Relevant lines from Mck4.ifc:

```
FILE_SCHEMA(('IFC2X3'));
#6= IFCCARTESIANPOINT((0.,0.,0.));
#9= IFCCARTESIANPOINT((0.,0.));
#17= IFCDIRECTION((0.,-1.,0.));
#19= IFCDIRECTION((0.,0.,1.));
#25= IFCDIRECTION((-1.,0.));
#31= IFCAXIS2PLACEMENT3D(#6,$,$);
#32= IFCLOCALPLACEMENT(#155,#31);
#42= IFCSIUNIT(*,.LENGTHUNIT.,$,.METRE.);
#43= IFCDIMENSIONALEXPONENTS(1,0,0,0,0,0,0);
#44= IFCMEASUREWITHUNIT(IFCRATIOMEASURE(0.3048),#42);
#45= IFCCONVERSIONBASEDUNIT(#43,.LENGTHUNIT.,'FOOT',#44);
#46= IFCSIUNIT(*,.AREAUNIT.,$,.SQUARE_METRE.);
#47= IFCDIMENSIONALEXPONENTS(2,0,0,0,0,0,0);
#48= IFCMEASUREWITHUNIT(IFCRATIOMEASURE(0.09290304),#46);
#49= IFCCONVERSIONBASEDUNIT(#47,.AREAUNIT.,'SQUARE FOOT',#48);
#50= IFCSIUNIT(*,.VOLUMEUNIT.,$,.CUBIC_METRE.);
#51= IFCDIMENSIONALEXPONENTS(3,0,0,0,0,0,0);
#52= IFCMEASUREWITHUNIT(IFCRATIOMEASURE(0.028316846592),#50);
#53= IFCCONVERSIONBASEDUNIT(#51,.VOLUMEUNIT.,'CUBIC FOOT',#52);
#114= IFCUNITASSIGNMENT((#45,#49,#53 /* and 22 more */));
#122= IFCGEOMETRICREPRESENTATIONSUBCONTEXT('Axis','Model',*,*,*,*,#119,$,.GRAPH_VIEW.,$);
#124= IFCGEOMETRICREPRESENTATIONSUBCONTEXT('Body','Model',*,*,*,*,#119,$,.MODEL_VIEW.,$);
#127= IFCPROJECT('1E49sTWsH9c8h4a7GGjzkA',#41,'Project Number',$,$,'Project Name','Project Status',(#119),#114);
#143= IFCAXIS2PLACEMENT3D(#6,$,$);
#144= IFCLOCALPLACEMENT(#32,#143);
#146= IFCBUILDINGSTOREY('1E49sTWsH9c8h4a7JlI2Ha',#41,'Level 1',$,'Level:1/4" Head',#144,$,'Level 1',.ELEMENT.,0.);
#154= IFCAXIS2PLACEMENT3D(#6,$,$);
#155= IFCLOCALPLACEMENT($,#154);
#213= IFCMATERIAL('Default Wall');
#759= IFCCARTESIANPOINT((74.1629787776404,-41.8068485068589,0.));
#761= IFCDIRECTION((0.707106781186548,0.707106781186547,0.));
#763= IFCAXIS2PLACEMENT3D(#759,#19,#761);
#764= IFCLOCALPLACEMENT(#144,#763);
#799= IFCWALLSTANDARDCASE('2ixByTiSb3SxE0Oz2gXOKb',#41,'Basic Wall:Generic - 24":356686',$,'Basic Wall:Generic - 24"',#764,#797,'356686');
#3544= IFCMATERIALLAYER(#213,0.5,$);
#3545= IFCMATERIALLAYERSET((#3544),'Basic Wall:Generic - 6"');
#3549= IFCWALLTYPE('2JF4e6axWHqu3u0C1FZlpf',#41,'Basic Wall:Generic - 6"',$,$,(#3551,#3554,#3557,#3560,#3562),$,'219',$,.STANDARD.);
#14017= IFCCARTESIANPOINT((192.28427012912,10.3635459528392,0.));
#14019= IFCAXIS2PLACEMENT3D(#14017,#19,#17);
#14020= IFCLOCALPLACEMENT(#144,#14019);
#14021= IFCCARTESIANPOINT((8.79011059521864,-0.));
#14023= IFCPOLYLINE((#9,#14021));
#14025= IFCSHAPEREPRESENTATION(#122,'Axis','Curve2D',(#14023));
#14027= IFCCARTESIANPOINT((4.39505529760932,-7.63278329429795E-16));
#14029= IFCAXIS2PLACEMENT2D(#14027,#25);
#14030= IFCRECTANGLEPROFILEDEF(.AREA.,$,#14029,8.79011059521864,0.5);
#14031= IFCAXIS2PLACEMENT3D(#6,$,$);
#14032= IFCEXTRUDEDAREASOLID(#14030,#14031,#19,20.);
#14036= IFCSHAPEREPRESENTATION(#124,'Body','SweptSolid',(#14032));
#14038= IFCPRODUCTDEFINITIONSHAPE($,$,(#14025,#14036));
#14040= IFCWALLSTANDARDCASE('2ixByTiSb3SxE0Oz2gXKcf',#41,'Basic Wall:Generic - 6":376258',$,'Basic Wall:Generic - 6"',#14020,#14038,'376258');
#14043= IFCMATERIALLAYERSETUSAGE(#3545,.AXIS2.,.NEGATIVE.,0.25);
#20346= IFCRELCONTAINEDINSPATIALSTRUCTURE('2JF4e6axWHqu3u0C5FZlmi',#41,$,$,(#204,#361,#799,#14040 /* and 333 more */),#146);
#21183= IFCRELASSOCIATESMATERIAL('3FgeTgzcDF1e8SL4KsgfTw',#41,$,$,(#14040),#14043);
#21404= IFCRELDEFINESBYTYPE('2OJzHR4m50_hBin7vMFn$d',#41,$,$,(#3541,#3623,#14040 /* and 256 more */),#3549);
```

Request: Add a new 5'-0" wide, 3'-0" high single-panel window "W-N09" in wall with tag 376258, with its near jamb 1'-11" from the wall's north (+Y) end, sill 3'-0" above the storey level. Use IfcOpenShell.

```python
import numpy as np
import ifcopenshell
import ifcopenshell.api.feature
import ifcopenshell.api.geometry
import ifcopenshell.api.root
import ifcopenshell.api.spatial
import ifcopenshell.api.type
import ifcopenshell.geom
import ifcopenshell.util.element
import ifcopenshell.util.placement
import ifcopenshell.util.representation
import ifcopenshell.util.shape
import ifcopenshell.util.unit

model = ifcopenshell.open("Mck4.ifc")
unit_scale = ifcopenshell.util.unit.calculate_unit_scale(model)
settings = ifcopenshell.geom.settings()


def volume(element):
    """Net volume in cubic metres, openings subtracted."""
    shape = ifcopenshell.geom.create_shape(settings, element)
    return ifcopenshell.util.shape.get_volume(shape.geometry)


wall = model.by_guid("2ixByTiSb3SxE0Oz2gXKcf")
storey = ifcopenshell.util.element.get_container(wall, ifc_class="IfcBuildingStorey")
context = ifcopenshell.util.representation.get_context(model, "Model", "Body", "MODEL_VIEW")
before = volume(wall)

width, height, from_end, sill = 1.524, 0.9144, 0.5842, 0.9144  # metres

# The wall runs along its own X axis, and the end named is its -X end.
wall_shape = ifcopenshell.geom.create_shape(settings, wall)
x, y, z = ifcopenshell.util.shape.get_vertices(wall_shape.geometry).T
start = x.min() + from_end
face, thickness = float(y.min()), float(y.max() - y.min())
wall_matrix = ifcopenshell.util.placement.get_local_placement(wall.ObjectPlacement)
level = ifcopenshell.util.placement.get_local_placement(storey.ObjectPlacement)[2, 3]


def in_wall(x, y):
    """Placement at x, y metres in the wall's axes, at sill height."""
    matrix = wall_matrix.copy()
    matrix[:, 3] = wall_matrix @ np.array([x / unit_scale, y / unit_scale, 0.0, 1.0])
    matrix[2, 3] = level + sill / unit_scale
    return matrix


# Opening: a box that overshoots both wall faces by 50 mm.
opening = ifcopenshell.api.root.create_entity(model, ifc_class="IfcOpeningElement")
box = ifcopenshell.api.geometry.add_wall_representation(
    model, context=context, length=width, height=height, thickness=thickness + 0.1
)
ifcopenshell.api.geometry.assign_representation(model, product=opening, representation=box)
ifcopenshell.api.geometry.edit_object_placement(model, product=opening, matrix=in_wall(start, face - 0.05), is_si=False)
ifcopenshell.api.feature.add_feature(model, feature=opening, element=wall)

window = ifcopenshell.api.root.create_entity(model, ifc_class="IfcWindow", name="W-N09")
window.OverallWidth, window.OverallHeight = width / unit_scale, height / unit_scale
body = ifcopenshell.api.geometry.add_window_representation(
    model,
    context=context,
    overall_width=window.OverallWidth,
    overall_height=window.OverallHeight,
    partition_type="SINGLE_PANEL",
)
ifcopenshell.api.geometry.assign_representation(model, product=window, representation=body)
ifcopenshell.api.spatial.assign_container(model, products=[window], relating_structure=storey)
fills = ifcopenshell.api.feature.add_filling(model, opening=opening, element=window)
fills.OwnerHistory = window.OwnerHistory  # required in IFC2X3

# IFC2X3 keeps the operation on the window style.
style = ifcopenshell.api.root.create_entity(model, ifc_class="IfcWindowStyle", name="W-N09")
style.OperationType, style.ConstructionType = "SINGLE_PANEL", "NOTDEFINED"
style.ParameterTakesPrecedence = style.Sizeable = False
ifcopenshell.api.type.assign_type(model, related_objects=[window], relating_type=style)

# Centre the window in the wall's thickness.
ifcopenshell.api.geometry.edit_object_placement(model, product=window, matrix=in_wall(start, face), is_si=False)
window_shape = ifcopenshell.geom.create_shape(settings, window)
depth = ifcopenshell.util.shape.get_vertices(window_shape.geometry)[:, 1]
offset = face + thickness / 2 - (depth.min() + depth.max()) / 2
ifcopenshell.api.geometry.edit_object_placement(model, product=window, matrix=in_wall(start, offset), is_si=False)

after = volume(wall)

print(f"wall volume {before:.3f} -> {after:.3f} m3")

model.write("Mck4-out.ifc")
```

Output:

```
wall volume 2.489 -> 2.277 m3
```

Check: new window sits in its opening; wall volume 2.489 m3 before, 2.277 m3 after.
